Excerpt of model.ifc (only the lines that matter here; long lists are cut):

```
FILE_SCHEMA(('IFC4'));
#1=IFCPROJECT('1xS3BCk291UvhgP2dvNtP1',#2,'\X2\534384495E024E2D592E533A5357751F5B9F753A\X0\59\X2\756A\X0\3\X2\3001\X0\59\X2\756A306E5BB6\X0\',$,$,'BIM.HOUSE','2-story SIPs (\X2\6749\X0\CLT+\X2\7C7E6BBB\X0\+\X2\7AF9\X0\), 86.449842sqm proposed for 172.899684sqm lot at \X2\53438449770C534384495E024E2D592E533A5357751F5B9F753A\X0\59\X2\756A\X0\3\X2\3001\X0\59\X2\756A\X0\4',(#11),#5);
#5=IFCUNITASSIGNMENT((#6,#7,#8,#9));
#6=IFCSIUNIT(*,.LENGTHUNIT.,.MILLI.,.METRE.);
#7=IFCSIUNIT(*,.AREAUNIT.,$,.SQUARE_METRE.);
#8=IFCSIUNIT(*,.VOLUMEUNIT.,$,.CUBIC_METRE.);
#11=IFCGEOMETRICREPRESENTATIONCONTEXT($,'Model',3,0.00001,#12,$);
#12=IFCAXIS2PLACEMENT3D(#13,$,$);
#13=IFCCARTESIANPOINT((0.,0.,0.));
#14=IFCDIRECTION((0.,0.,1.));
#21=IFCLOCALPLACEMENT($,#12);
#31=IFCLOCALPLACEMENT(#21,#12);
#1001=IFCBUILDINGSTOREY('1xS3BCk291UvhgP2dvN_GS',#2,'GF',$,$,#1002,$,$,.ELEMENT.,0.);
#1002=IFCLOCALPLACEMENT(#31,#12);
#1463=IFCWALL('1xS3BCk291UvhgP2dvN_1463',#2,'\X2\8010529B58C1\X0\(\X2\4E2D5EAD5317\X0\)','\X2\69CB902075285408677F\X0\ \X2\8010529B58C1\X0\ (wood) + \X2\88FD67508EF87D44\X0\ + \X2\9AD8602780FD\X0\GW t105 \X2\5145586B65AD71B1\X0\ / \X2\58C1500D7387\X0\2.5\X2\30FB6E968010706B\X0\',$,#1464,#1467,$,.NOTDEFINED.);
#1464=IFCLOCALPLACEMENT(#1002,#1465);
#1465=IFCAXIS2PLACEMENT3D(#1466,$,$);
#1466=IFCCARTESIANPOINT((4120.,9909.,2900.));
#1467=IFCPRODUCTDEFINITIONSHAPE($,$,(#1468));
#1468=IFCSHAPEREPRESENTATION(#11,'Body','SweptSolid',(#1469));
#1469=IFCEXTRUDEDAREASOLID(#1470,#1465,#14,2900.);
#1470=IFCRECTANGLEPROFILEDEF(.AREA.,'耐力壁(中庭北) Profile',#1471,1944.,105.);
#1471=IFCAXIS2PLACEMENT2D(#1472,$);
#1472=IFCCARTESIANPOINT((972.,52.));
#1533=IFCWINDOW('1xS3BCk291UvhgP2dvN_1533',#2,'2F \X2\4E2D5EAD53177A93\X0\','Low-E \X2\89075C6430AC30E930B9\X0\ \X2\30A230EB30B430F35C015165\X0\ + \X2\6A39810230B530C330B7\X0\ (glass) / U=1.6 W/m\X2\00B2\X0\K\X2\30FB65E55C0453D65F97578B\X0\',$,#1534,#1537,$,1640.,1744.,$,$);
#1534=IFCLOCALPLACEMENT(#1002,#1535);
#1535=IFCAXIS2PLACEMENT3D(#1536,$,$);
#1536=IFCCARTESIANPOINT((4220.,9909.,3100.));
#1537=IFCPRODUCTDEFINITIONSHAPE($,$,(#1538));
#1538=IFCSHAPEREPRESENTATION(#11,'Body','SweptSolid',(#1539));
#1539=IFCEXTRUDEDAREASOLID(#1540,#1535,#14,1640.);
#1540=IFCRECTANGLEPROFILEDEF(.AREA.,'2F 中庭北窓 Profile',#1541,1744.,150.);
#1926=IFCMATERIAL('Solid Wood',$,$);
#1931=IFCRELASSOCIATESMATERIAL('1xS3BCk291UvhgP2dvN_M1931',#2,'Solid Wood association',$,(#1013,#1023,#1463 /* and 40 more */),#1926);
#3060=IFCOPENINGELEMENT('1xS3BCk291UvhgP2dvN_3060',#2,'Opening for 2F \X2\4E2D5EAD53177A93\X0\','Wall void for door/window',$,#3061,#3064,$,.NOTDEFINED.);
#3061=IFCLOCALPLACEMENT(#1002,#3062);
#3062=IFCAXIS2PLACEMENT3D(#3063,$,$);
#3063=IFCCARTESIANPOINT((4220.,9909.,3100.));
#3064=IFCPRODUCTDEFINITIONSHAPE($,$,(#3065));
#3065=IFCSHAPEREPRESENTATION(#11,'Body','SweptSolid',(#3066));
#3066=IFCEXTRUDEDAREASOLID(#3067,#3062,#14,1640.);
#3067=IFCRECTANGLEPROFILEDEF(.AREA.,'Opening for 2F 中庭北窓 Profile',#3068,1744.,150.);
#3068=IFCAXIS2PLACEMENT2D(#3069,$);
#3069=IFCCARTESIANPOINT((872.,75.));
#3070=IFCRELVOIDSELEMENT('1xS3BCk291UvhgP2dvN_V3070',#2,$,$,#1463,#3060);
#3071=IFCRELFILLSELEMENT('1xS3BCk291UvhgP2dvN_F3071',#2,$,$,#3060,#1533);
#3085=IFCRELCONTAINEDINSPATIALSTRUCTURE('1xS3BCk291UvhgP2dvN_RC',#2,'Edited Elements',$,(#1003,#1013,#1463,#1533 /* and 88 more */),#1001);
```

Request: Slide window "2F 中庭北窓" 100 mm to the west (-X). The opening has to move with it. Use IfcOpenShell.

```python
import ifcopenshell
import ifcopenshell.api.geometry
import ifcopenshell.util.placement
import ifcopenshell.util.unit

model = ifcopenshell.open("model.ifc")
unit_scale = ifcopenshell.util.unit.calculate_unit_scale(model)

window = model.by_id(1533)
opening = window.FillsVoids[0].RelatingOpeningElement
wall = opening.VoidsElements[0].RelatingBuildingElement

wall_matrix = ifcopenshell.util.placement.get_local_placement(wall.ObjectPlacement)
shift = wall_matrix[:3, 0] * -0.1 / unit_scale
before = ifcopenshell.util.placement.get_local_placement(window.ObjectPlacement)[:3, 3].copy()

# The window is not placed relative to its opening, so move both.
for product in (opening, window):
    matrix = ifcopenshell.util.placement.get_local_placement(product.ObjectPlacement)
    matrix[:3, 3] += shift
    ifcopenshell.api.geometry.edit_object_placement(model, product=product, matrix=matrix, is_si=False)

after = ifcopenshell.util.placement.get_local_placement(window.ObjectPlacement)[:3, 3]
print("window moved by", (after - before).round(3) + 0.0)

model.write("model_rev.ifc")
```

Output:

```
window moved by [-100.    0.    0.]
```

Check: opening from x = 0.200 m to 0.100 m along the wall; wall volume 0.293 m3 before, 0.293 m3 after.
